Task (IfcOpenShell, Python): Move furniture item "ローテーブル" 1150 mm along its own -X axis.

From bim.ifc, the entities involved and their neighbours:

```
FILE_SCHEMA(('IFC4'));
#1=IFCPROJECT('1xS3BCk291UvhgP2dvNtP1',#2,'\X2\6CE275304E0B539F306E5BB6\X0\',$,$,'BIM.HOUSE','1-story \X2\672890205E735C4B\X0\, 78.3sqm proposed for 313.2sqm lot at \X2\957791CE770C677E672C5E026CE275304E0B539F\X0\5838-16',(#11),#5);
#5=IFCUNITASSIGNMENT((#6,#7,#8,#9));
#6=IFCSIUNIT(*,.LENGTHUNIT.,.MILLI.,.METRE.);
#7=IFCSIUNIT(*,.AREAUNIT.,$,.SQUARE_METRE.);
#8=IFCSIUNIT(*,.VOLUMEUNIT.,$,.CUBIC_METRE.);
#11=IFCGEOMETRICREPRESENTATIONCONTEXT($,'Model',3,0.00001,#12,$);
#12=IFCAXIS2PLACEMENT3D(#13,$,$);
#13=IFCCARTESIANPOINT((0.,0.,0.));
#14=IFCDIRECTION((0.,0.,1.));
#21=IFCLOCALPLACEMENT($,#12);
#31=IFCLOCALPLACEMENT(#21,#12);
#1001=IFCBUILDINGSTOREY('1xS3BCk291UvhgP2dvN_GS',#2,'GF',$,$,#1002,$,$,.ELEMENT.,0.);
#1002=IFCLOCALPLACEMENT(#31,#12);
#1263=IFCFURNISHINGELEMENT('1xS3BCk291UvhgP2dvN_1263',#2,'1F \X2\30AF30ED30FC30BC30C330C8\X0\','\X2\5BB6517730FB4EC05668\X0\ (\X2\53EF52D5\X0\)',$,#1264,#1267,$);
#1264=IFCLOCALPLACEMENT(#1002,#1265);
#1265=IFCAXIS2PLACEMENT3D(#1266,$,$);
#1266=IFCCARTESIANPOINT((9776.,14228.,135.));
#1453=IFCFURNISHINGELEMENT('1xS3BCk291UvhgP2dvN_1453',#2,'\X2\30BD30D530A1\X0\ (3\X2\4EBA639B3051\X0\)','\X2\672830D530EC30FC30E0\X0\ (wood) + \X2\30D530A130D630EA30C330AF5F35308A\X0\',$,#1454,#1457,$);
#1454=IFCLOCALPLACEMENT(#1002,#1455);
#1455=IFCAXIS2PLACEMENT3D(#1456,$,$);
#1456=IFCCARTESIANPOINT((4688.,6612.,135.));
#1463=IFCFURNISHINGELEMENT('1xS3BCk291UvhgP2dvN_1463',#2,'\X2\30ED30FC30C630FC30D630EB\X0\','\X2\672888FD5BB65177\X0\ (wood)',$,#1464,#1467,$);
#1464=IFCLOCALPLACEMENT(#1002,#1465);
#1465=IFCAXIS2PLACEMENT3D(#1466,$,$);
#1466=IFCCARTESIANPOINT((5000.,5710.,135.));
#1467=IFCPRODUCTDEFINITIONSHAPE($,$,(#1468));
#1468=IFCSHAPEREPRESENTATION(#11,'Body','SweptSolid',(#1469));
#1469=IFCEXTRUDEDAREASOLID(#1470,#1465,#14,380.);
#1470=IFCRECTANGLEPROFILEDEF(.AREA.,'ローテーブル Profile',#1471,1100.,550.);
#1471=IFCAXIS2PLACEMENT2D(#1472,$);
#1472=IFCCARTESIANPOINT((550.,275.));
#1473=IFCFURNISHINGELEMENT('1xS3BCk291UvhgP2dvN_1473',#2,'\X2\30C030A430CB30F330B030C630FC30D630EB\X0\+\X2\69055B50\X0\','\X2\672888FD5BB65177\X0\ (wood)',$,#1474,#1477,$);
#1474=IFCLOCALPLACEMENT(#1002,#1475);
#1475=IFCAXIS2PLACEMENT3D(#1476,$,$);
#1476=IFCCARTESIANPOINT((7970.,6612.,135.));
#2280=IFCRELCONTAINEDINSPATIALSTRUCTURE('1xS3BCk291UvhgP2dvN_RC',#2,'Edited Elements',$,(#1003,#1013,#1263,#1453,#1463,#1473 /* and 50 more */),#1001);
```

```python
import ifcopenshell
import ifcopenshell.api.geometry
import ifcopenshell.util.placement
import ifcopenshell.util.unit

model = ifcopenshell.open("bim.ifc")
unit_scale = ifcopenshell.util.unit.calculate_unit_scale(model)

item = model.by_id(1463)
matrix = ifcopenshell.util.placement.get_local_placement(item.ObjectPlacement)
matrix[:3, 3] -= matrix[:3, 0] * 1.15 / unit_scale
ifcopenshell.api.geometry.edit_object_placement(model, product=item, matrix=matrix, is_si=False)

print(ifcopenshell.util.placement.get_local_placement(item.ObjectPlacement).round(3) + 0.0)

model.write("bim-out.ifc")
```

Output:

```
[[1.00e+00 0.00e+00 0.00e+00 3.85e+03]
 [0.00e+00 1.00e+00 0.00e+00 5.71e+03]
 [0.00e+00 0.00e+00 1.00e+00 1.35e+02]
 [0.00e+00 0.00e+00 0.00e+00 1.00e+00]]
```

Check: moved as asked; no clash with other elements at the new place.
